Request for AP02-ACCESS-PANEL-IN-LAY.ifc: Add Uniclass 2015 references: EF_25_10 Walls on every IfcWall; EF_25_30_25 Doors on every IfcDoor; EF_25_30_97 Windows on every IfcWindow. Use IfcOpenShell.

First a look at what the model holds.

```python
import ifcopenshell

model = ifcopenshell.open("AP02-ACCESS-PANEL-IN-LAY.ifc")
print(model.schema)
print("classifications:", [c.Name for c in model.by_type("IfcClassification")])
for ifc_class in ("IfcDoor", "IfcRoof", "IfcStair", "IfcWall", "IfcWindow"):
    print(ifc_class, len(model.by_type(ifc_class)))
```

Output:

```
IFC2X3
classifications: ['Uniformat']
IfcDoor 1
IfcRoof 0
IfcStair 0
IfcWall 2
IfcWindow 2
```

```python
import ifcopenshell
import ifcopenshell.api.classification

model = ifcopenshell.open("AP02-ACCESS-PANEL-IN-LAY.ifc")

# IFC2X3 requires Source and Edition and has no link from the project to the system.
system = model.create_entity("IfcClassification", Source="NBS", Edition="2015", Name="Uniclass 2015")

codes = {
    "IfcWall": ("EF_25_10", "Walls"),
    "IfcDoor": ("EF_25_30_25", "Doors"),
    "IfcWindow": ("EF_25_30_97", "Windows"),
}
for ifc_class, (code, name) in codes.items():
    products = model.by_type(ifc_class)
    ifcopenshell.api.classification.add_reference(
        model, products=products, classification=system, identification=code, name=name
    )
    print(code, len(products))

model.write("AP02-ACCESS-PANEL-IN-LAY-out.ifc")
```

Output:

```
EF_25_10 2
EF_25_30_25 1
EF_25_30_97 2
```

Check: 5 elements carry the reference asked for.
